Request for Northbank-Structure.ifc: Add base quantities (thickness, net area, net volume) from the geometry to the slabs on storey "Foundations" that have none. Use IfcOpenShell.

First a look at what the model holds.

```python
import ifcopenshell
import ifcopenshell.util.element
import ifcopenshell.util.unit

model = ifcopenshell.open("Northbank-Structure.ifc")
print(model.schema)
for unit_type in ("LENGTHUNIT", "AREAUNIT", "VOLUMEUNIT"):
    print(unit_type, ifcopenshell.util.unit.calculate_unit_scale(model, unit_type))
storey = next(s for s in model.by_type("IfcBuildingStorey") if s.Name == "Foundations")
slabs = [e for e in ifcopenshell.util.element.get_decomposition(storey) if e.is_a("IfcSlab")]
for e in sorted(slabs, key=lambda e: e.id()):
    print(e.id(), e.is_a(), e.Name, list(ifcopenshell.util.element.get_psets(e, qtos_only=True)), sep=" | ")
```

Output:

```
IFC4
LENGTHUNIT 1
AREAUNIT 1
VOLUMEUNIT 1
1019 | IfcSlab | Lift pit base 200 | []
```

```python
import ifcopenshell
import ifcopenshell.api.pset
import ifcopenshell.geom
import ifcopenshell.util.element
import ifcopenshell.util.shape
import ifcopenshell.util.unit

model = ifcopenshell.open("Northbank-Structure.ifc")
unit_scale = ifcopenshell.util.unit.calculate_unit_scale(model)
area_scale = ifcopenshell.util.unit.calculate_unit_scale(model, "AREAUNIT")
volume_scale = ifcopenshell.util.unit.calculate_unit_scale(model, "VOLUMEUNIT")
settings = ifcopenshell.geom.settings()

storey = next(s for s in model.by_type("IfcBuildingStorey") if s.Name == "Foundations")
slabs = [e for e in ifcopenshell.util.element.get_decomposition(storey) if e.is_a("IfcSlab")]

for e in sorted(slabs, key=lambda e: e.id()):
    if ifcopenshell.util.element.get_psets(e, qtos_only=True, should_inherit=False):
        continue
    # Geometry comes back in metres, in the element's own axes.
    shape = ifcopenshell.geom.create_shape(settings, e)
    values = {
        "Width": ifcopenshell.util.shape.get_z(shape.geometry) / unit_scale,
        "NetArea": ifcopenshell.util.shape.get_footprint_area(shape.geometry) / area_scale,
        "NetVolume": ifcopenshell.util.shape.get_volume(shape.geometry) / volume_scale,
    }
    qto = ifcopenshell.api.pset.add_qto(model, product=e, name="Qto_SlabBaseQuantities")
    ifcopenshell.api.pset.edit_qto(model, qto=qto, properties=values)
    print(e.id(), {k: round(v, 3) for k, v in values.items()})

model.write("Northbank-Structure_v2.ifc")
```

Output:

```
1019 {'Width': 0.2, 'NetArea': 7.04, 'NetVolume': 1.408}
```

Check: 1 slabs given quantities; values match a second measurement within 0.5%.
